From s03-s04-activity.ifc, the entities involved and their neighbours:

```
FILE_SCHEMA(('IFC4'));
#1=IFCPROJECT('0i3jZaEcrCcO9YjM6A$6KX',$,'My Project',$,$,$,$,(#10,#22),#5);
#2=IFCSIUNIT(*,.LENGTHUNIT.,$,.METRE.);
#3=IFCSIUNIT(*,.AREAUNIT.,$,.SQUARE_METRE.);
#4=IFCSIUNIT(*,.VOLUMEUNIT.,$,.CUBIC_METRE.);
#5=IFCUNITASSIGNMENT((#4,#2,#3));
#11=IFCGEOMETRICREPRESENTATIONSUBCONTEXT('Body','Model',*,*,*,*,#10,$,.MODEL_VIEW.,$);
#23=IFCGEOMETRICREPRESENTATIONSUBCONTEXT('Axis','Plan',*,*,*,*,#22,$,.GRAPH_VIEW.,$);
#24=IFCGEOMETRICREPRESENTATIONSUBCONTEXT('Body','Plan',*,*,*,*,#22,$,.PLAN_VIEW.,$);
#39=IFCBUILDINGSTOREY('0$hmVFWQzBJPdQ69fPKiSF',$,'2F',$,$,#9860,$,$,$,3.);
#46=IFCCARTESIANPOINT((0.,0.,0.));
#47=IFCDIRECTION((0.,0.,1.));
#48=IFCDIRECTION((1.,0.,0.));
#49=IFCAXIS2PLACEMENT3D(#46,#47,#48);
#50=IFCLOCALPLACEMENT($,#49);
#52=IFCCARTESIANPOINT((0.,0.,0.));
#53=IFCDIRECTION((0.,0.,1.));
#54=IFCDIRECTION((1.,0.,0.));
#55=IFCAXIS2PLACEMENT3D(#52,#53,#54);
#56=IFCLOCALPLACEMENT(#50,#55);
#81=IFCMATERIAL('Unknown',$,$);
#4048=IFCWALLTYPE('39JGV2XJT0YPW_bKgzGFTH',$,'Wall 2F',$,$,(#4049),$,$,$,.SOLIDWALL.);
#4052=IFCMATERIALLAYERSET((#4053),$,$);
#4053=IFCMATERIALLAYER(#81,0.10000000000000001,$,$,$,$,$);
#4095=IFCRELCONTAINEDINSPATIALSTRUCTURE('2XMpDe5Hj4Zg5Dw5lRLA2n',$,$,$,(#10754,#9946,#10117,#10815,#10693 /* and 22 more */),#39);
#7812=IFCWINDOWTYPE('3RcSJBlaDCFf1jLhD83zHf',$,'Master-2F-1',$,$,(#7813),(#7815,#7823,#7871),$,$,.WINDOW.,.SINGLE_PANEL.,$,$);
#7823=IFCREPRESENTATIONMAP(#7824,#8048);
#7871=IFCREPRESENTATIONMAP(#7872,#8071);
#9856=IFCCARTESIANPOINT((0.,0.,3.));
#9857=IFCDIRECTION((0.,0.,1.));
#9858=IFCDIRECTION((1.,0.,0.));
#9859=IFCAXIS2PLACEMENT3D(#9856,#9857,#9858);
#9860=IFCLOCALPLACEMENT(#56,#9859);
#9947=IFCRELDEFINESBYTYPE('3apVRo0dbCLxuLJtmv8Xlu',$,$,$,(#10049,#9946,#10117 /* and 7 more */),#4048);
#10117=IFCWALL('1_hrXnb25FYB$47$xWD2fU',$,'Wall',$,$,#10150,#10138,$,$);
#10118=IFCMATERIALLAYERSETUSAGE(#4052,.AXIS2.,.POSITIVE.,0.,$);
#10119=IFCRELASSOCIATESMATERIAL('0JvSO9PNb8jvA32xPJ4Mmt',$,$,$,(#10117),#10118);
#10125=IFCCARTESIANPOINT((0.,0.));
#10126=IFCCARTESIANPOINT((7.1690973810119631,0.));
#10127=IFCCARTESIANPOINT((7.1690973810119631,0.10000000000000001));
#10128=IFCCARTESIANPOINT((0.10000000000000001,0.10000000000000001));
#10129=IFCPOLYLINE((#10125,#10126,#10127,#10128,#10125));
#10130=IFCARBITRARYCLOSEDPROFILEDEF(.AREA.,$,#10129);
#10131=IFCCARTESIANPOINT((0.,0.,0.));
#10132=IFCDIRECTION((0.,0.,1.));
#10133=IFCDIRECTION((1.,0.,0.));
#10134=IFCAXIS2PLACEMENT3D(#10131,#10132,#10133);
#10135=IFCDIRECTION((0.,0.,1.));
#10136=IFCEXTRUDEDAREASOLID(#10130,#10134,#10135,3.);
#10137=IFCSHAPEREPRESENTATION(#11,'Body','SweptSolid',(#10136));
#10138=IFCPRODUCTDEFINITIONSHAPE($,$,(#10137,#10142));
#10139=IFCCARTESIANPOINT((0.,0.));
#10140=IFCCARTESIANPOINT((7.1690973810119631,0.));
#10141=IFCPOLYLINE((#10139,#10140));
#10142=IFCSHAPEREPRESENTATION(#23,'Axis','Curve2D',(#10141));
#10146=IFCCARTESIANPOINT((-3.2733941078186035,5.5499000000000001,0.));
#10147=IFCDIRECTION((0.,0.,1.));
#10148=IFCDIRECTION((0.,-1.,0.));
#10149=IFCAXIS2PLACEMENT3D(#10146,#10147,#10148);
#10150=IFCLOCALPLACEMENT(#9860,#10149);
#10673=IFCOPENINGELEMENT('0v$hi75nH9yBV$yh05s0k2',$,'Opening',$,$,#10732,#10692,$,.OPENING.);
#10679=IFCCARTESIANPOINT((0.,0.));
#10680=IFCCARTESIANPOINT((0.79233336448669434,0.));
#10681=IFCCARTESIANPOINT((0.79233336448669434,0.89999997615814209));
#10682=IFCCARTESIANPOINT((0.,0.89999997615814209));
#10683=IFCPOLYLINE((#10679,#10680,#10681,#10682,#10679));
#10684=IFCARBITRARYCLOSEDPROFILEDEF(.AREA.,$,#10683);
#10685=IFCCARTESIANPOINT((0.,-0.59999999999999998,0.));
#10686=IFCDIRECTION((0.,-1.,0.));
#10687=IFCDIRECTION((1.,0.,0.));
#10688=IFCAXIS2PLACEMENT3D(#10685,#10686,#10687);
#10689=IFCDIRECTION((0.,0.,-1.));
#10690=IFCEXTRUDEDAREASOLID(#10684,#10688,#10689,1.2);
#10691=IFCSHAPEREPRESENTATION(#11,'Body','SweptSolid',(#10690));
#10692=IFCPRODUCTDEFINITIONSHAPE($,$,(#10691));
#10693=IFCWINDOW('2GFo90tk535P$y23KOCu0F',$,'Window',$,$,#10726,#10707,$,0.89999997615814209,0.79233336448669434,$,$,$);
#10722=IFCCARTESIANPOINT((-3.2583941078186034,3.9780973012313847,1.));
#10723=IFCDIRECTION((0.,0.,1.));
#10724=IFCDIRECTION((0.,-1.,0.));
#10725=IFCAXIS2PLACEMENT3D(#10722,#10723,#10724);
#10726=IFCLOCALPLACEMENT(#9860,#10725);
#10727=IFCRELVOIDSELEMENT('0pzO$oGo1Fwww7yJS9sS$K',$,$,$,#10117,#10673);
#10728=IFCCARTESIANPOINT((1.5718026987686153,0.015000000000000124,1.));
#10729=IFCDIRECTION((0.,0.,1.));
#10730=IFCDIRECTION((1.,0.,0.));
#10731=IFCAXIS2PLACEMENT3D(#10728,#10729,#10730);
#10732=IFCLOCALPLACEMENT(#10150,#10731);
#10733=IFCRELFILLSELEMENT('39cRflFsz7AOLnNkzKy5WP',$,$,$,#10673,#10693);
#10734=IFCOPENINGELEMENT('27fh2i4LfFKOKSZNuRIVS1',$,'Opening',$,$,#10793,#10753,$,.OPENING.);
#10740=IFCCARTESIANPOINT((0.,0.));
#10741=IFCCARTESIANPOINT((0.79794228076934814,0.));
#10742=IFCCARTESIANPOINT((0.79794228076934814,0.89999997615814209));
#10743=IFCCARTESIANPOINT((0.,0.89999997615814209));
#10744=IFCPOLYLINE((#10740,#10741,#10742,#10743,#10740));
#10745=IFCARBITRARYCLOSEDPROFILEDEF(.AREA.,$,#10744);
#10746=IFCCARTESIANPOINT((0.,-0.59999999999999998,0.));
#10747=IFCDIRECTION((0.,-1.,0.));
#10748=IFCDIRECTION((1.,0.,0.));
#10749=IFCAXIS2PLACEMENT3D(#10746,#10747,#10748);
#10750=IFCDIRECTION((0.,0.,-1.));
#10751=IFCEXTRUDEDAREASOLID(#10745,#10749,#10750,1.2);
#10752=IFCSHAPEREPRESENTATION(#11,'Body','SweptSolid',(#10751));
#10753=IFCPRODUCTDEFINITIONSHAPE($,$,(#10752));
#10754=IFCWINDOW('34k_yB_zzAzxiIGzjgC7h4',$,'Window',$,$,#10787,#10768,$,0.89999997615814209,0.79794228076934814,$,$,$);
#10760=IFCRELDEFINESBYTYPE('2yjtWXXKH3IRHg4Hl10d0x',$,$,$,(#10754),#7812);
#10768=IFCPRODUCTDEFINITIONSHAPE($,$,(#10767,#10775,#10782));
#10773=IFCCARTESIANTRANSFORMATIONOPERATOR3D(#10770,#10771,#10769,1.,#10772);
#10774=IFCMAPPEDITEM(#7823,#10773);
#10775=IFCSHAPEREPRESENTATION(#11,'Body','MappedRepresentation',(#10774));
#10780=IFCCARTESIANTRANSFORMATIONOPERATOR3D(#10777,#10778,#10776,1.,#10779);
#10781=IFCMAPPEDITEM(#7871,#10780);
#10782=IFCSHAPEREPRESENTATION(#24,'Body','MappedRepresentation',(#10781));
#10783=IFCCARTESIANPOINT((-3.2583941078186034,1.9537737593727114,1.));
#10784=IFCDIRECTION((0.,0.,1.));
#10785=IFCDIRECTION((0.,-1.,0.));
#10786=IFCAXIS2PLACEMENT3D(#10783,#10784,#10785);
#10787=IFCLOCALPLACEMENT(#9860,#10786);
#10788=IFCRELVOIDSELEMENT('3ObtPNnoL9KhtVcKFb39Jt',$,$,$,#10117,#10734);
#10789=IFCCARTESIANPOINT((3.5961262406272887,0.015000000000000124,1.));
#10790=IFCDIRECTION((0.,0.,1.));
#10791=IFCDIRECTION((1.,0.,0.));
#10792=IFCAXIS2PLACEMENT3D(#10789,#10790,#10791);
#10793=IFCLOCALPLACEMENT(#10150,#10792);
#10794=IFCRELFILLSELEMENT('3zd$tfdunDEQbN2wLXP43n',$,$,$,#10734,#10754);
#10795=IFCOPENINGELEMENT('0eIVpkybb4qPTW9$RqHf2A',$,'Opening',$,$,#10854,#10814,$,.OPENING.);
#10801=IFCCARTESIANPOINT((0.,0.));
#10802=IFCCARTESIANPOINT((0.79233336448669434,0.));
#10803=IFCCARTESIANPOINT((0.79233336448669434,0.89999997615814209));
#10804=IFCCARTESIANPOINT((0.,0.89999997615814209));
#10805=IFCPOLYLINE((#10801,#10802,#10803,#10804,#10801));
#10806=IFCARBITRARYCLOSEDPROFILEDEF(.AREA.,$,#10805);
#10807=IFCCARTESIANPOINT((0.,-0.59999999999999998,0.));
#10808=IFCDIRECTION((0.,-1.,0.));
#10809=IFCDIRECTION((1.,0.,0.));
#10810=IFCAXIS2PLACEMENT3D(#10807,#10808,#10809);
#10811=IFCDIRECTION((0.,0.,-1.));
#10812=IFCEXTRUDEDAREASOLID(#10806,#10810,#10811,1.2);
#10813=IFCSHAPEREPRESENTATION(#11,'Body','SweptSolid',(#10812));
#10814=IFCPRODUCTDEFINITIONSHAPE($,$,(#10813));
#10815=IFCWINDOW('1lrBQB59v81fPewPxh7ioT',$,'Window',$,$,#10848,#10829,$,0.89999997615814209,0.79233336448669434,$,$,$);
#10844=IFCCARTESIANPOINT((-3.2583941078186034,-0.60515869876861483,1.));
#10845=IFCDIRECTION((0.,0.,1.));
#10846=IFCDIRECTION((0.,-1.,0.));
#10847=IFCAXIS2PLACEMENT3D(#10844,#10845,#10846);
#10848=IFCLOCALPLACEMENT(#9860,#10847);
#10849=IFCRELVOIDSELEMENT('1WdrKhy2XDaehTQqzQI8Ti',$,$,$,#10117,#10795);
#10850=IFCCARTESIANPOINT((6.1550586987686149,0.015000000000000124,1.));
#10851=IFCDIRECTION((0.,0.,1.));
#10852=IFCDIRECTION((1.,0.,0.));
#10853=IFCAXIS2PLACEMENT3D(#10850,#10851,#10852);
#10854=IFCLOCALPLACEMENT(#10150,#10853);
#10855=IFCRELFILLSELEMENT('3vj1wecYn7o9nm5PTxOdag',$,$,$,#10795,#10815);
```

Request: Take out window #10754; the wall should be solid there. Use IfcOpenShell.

```python
import ifcopenshell
import ifcopenshell.api.feature
import ifcopenshell.api.root
import ifcopenshell.geom
import ifcopenshell.util.shape

model = ifcopenshell.open("s03-s04-activity.ifc")
settings = ifcopenshell.geom.settings()


def volume(element):
    """Net volume in cubic metres, openings subtracted."""
    shape = ifcopenshell.geom.create_shape(settings, element)
    return ifcopenshell.util.shape.get_volume(shape.geometry)


window = model.by_guid("34k_yB_zzAzxiIGzjgC7h4")
opening = window.FillsVoids[0].RelatingOpeningElement
wall = opening.VoidsElements[0].RelatingBuildingElement
before = volume(wall)

ifcopenshell.api.root.remove_product(model, product=window)
ifcopenshell.api.feature.remove_feature(model, feature=opening)

after = volume(wall)

print(f"wall volume {before:.3f} -> {after:.3f} m3")

model.write("s03-s04-activity_rev.ifc")
```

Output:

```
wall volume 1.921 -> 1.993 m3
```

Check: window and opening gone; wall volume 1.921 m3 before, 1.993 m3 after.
